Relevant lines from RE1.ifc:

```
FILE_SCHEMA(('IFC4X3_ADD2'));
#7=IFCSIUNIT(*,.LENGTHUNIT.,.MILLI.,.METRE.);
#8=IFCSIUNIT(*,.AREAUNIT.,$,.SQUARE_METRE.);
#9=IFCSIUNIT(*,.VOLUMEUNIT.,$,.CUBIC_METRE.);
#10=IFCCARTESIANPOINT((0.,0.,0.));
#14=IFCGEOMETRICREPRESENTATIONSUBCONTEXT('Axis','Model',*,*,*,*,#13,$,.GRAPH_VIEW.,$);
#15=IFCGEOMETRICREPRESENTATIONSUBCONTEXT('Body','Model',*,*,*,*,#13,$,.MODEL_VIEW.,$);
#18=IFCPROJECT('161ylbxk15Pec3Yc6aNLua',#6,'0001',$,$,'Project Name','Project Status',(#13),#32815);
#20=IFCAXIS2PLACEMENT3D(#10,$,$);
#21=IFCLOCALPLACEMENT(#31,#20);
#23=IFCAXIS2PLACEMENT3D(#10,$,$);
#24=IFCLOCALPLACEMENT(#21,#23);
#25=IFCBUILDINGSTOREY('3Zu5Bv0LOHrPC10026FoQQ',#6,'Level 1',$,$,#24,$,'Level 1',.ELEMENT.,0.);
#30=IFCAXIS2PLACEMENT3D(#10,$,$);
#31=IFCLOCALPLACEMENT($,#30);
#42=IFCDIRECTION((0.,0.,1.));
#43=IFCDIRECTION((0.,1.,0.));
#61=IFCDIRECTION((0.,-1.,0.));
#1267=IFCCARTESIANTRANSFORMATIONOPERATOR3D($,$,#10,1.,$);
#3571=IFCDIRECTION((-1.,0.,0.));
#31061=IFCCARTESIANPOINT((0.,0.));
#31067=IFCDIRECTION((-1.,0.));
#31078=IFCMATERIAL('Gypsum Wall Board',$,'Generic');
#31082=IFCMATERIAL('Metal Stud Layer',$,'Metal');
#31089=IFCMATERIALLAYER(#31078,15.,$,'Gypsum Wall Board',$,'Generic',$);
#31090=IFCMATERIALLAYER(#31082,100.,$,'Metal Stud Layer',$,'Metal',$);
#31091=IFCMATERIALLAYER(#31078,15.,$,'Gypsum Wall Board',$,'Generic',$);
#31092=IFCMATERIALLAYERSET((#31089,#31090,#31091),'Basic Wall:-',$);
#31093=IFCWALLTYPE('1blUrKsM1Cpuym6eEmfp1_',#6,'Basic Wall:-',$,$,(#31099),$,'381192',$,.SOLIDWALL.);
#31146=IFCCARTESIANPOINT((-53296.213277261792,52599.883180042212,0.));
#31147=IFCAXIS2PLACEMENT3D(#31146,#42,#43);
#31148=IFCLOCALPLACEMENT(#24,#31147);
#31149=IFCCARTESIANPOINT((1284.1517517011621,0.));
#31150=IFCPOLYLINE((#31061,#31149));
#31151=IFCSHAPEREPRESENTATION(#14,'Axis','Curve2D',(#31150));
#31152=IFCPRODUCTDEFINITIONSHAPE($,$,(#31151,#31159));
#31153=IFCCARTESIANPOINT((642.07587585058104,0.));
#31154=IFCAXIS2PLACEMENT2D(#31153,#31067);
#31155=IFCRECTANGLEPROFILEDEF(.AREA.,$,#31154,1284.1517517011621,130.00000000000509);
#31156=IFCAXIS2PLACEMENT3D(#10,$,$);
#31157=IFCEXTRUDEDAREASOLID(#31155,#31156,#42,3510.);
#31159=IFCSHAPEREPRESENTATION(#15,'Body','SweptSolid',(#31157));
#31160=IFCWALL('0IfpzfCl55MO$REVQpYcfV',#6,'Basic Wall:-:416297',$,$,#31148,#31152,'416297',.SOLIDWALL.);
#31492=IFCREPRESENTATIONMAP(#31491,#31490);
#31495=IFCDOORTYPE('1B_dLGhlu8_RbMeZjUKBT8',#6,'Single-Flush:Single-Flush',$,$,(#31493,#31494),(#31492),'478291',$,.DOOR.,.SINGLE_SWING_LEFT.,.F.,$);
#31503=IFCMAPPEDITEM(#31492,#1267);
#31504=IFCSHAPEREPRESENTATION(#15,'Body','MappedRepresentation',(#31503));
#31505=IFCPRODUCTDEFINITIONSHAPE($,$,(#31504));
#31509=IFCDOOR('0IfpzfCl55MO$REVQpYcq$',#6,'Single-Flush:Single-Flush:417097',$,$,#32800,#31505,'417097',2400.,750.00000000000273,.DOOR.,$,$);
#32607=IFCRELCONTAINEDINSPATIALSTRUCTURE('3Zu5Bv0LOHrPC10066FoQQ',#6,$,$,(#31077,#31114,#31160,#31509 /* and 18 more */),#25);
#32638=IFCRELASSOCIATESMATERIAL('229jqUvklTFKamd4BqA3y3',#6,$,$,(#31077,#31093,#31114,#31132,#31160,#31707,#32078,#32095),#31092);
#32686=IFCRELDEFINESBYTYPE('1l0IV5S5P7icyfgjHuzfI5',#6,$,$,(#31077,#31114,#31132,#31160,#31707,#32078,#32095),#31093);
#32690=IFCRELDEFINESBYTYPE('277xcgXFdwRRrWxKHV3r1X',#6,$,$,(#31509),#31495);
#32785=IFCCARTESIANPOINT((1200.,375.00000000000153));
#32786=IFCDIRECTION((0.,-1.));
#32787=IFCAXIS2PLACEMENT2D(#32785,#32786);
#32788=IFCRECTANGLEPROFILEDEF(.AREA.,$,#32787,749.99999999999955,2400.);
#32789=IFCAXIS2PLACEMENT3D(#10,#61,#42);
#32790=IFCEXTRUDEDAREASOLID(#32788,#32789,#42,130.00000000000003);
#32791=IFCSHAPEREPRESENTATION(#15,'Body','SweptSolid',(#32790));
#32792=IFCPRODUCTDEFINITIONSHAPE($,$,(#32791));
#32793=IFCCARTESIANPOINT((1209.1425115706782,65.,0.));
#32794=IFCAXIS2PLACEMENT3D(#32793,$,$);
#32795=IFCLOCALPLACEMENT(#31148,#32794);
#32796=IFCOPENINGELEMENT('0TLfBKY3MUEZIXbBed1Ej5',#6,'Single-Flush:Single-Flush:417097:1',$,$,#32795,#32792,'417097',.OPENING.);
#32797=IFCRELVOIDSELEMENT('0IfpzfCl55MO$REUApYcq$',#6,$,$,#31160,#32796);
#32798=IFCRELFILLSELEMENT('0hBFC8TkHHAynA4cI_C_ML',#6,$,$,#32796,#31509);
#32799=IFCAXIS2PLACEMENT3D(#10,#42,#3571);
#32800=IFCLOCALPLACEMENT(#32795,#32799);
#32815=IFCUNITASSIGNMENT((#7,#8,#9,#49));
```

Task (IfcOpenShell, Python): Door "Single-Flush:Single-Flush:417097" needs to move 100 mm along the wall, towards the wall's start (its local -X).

```python
import ifcopenshell
import ifcopenshell.api.geometry
import ifcopenshell.util.placement
import ifcopenshell.util.unit

model = ifcopenshell.open("RE1.ifc")
unit_scale = ifcopenshell.util.unit.calculate_unit_scale(model)

door = model.by_id(31509)
opening = door.FillsVoids[0].RelatingOpeningElement
wall = opening.VoidsElements[0].RelatingBuildingElement

wall_matrix = ifcopenshell.util.placement.get_local_placement(wall.ObjectPlacement)
shift = wall_matrix[:3, 0] * -0.1 / unit_scale
before = ifcopenshell.util.placement.get_local_placement(door.ObjectPlacement)[:3, 3].copy()

# The door is placed relative to its opening, so it follows when the opening moves.
matrix = ifcopenshell.util.placement.get_local_placement(opening.ObjectPlacement)
matrix[:3, 3] += shift
ifcopenshell.api.geometry.edit_object_placement(
    model, product=opening, matrix=matrix, is_si=False, should_transform_children=True
)

after = ifcopenshell.util.placement.get_local_placement(door.ObjectPlacement)[:3, 3]
print("door moved by", (after - before).round(3) + 0.0)

model.write("RE1_updated.ifc")
```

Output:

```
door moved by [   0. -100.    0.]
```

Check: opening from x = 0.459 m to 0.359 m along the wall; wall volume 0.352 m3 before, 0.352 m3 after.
